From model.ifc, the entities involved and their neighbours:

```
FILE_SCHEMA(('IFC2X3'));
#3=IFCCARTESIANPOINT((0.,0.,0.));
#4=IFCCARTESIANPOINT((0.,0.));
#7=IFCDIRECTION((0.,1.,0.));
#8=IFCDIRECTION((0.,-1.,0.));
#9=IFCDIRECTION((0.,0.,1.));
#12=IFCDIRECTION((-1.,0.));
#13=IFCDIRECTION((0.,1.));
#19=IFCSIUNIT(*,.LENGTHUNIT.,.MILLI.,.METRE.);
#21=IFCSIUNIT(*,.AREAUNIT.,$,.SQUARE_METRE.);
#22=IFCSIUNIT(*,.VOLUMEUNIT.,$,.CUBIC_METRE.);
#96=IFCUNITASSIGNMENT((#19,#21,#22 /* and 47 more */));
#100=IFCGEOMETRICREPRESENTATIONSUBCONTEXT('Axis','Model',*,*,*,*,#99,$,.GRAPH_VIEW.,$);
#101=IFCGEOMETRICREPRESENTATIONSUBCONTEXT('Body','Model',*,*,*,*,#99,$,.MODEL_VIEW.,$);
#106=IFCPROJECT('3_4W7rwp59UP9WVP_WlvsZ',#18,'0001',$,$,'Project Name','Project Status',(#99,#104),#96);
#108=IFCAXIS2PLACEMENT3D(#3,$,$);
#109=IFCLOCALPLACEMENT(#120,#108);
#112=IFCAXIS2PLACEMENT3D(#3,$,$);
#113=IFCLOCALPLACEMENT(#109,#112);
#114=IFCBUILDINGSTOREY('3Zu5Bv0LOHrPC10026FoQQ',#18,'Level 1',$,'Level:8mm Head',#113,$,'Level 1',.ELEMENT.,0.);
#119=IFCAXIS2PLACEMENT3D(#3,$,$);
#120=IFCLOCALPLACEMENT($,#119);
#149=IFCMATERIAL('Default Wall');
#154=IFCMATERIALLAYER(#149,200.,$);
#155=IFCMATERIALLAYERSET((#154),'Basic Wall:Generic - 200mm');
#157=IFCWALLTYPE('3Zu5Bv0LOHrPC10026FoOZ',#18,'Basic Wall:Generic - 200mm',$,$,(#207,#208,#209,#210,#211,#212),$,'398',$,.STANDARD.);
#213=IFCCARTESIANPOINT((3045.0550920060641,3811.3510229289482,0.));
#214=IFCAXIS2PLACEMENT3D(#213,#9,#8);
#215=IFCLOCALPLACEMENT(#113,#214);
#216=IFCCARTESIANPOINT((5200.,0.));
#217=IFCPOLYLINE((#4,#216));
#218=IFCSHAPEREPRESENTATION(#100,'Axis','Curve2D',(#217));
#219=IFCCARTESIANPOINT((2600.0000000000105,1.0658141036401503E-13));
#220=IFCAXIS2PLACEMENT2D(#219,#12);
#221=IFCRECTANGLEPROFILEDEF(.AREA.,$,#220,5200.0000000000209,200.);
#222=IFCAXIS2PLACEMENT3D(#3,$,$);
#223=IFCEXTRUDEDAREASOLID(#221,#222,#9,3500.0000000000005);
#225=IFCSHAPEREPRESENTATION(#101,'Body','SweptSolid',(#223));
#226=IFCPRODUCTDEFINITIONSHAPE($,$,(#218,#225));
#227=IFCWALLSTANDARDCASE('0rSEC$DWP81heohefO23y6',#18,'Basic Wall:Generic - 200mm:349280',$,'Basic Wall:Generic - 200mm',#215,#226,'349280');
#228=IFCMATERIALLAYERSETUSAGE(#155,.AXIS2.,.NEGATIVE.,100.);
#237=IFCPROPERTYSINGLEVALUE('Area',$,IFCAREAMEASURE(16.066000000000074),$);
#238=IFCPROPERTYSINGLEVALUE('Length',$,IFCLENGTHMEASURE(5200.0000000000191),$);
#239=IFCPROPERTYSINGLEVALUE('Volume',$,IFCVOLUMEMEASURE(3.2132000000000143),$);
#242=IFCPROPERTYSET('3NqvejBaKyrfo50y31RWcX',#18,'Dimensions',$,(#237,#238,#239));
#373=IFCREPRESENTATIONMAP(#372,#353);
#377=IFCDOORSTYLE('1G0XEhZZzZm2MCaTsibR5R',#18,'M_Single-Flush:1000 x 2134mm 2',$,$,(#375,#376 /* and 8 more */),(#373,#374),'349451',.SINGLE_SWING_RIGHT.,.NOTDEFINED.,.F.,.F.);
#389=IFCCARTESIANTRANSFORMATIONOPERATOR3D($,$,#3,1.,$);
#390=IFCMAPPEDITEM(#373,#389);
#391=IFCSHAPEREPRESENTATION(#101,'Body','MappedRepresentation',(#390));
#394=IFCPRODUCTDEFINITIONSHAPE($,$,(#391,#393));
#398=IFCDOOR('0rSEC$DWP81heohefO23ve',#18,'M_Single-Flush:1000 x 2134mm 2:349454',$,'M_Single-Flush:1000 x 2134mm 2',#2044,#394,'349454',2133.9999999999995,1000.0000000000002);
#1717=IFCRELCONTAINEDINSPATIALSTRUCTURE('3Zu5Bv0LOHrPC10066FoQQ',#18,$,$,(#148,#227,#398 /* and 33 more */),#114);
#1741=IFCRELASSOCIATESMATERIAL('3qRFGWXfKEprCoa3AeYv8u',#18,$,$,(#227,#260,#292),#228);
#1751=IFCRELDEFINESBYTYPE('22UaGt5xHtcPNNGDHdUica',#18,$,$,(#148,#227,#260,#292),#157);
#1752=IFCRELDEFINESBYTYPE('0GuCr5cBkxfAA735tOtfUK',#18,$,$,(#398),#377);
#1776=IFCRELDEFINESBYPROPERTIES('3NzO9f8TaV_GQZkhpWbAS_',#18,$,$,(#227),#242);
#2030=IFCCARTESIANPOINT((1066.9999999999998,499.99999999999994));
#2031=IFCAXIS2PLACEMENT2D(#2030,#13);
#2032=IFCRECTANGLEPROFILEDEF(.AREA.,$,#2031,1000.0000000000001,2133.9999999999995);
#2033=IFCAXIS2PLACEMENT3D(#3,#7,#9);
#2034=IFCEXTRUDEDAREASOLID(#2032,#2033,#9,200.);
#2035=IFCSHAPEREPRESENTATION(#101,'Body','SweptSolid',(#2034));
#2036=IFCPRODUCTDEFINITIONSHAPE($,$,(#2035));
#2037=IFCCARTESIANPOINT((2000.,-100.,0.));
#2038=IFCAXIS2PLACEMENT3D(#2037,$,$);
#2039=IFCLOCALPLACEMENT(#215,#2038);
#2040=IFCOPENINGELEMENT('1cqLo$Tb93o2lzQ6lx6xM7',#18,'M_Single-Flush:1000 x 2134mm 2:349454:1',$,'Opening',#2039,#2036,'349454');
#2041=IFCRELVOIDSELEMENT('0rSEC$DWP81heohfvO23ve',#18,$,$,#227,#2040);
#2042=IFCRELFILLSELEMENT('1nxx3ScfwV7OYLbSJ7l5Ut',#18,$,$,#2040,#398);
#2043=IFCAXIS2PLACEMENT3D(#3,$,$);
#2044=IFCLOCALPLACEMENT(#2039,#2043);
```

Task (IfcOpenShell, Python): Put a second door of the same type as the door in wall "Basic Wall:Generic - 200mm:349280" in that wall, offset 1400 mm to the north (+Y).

```python
import ifcopenshell
import ifcopenshell.api.feature
import ifcopenshell.api.geometry
import ifcopenshell.api.pset
import ifcopenshell.api.root
import ifcopenshell.geom
import ifcopenshell.util.element
import ifcopenshell.util.placement
import ifcopenshell.util.shape
import ifcopenshell.util.unit

model = ifcopenshell.open("model.ifc")
unit_scale = ifcopenshell.util.unit.calculate_unit_scale(model)
area_scale = ifcopenshell.util.unit.calculate_unit_scale(model, "AREAUNIT")
volume_scale = ifcopenshell.util.unit.calculate_unit_scale(model, "VOLUMEUNIT")
settings = ifcopenshell.geom.settings()


def volume(element):
    """Net volume in cubic metres, openings subtracted."""
    shape = ifcopenshell.geom.create_shape(settings, element)
    return ifcopenshell.util.shape.get_volume(shape.geometry)


def reuse_history(source, copy):
    """copy_class also copies each property set's owner history, people and application; keep the originals."""
    for rel in copy.IsDefinedBy:
        if rel.is_a("IfcRelDefinesByProperties") and (history := rel.RelatingPropertyDefinition.OwnerHistory):
            rel.RelatingPropertyDefinition.OwnerHistory = source.OwnerHistory
            ifcopenshell.util.element.remove_deep2(model, history)


door = model.by_id(398)
opening = door.FillsVoids[0].RelatingOpeningElement
wall = opening.VoidsElements[0].RelatingBuildingElement
before = volume(wall)
shift = ifcopenshell.util.placement.get_local_placement(wall.ObjectPlacement)[:3, 0] * -1.4 / unit_scale

# copy_class copies the void relationship, type, container and properties, but no geometry.
new_opening = ifcopenshell.api.root.copy_class(model, product=opening)
new_opening.Representation = ifcopenshell.util.element.copy_deep(
    model, opening.Representation, exclude=["IfcGeometricRepresentationContext", "IfcRepresentationMap"]
)
new_opening.Name = "M_Single-Flush:1000 x 2134mm 2"
new_opening.Tag = None
new_door = ifcopenshell.api.root.copy_class(model, product=door)
new_door.Representation = ifcopenshell.util.element.copy_deep(
    model, door.Representation, exclude=["IfcGeometricRepresentationContext", "IfcRepresentationMap"]
)
new_door.Name = "M_Single-Flush:1000 x 2134mm 2"
new_door.Tag = None
reuse_history(door, new_door)
fills = ifcopenshell.api.feature.add_filling(model, opening=new_opening, element=new_door)
fills.OwnerHistory = new_door.OwnerHistory  # required in IFC2X3

for old, new in ((opening, new_opening), (door, new_door)):
    matrix = ifcopenshell.util.placement.get_local_placement(old.ObjectPlacement)
    matrix[:3, 3] += shift
    ifcopenshell.api.geometry.edit_object_placement(model, product=new, matrix=matrix, is_si=False)

after = volume(wall)
thickness = 0.2  # wall thickness in metres

# Update the wall's stored quantities.
pset = model.by_id(ifcopenshell.util.element.get_pset(wall, "Dimensions", should_inherit=False)["id"])
ifcopenshell.api.pset.edit_pset(model, pset=pset, properties={
    "Area": model.create_entity("IfcAreaMeasure", after / thickness / area_scale),
    "Volume": model.create_entity("IfcVolumeMeasure", after / volume_scale),
})

print(f"wall volume {before:.3f} -> {after:.3f} m3")

model.write("model-out.ifc")
```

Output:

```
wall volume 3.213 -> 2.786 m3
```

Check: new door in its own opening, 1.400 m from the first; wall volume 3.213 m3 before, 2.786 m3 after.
